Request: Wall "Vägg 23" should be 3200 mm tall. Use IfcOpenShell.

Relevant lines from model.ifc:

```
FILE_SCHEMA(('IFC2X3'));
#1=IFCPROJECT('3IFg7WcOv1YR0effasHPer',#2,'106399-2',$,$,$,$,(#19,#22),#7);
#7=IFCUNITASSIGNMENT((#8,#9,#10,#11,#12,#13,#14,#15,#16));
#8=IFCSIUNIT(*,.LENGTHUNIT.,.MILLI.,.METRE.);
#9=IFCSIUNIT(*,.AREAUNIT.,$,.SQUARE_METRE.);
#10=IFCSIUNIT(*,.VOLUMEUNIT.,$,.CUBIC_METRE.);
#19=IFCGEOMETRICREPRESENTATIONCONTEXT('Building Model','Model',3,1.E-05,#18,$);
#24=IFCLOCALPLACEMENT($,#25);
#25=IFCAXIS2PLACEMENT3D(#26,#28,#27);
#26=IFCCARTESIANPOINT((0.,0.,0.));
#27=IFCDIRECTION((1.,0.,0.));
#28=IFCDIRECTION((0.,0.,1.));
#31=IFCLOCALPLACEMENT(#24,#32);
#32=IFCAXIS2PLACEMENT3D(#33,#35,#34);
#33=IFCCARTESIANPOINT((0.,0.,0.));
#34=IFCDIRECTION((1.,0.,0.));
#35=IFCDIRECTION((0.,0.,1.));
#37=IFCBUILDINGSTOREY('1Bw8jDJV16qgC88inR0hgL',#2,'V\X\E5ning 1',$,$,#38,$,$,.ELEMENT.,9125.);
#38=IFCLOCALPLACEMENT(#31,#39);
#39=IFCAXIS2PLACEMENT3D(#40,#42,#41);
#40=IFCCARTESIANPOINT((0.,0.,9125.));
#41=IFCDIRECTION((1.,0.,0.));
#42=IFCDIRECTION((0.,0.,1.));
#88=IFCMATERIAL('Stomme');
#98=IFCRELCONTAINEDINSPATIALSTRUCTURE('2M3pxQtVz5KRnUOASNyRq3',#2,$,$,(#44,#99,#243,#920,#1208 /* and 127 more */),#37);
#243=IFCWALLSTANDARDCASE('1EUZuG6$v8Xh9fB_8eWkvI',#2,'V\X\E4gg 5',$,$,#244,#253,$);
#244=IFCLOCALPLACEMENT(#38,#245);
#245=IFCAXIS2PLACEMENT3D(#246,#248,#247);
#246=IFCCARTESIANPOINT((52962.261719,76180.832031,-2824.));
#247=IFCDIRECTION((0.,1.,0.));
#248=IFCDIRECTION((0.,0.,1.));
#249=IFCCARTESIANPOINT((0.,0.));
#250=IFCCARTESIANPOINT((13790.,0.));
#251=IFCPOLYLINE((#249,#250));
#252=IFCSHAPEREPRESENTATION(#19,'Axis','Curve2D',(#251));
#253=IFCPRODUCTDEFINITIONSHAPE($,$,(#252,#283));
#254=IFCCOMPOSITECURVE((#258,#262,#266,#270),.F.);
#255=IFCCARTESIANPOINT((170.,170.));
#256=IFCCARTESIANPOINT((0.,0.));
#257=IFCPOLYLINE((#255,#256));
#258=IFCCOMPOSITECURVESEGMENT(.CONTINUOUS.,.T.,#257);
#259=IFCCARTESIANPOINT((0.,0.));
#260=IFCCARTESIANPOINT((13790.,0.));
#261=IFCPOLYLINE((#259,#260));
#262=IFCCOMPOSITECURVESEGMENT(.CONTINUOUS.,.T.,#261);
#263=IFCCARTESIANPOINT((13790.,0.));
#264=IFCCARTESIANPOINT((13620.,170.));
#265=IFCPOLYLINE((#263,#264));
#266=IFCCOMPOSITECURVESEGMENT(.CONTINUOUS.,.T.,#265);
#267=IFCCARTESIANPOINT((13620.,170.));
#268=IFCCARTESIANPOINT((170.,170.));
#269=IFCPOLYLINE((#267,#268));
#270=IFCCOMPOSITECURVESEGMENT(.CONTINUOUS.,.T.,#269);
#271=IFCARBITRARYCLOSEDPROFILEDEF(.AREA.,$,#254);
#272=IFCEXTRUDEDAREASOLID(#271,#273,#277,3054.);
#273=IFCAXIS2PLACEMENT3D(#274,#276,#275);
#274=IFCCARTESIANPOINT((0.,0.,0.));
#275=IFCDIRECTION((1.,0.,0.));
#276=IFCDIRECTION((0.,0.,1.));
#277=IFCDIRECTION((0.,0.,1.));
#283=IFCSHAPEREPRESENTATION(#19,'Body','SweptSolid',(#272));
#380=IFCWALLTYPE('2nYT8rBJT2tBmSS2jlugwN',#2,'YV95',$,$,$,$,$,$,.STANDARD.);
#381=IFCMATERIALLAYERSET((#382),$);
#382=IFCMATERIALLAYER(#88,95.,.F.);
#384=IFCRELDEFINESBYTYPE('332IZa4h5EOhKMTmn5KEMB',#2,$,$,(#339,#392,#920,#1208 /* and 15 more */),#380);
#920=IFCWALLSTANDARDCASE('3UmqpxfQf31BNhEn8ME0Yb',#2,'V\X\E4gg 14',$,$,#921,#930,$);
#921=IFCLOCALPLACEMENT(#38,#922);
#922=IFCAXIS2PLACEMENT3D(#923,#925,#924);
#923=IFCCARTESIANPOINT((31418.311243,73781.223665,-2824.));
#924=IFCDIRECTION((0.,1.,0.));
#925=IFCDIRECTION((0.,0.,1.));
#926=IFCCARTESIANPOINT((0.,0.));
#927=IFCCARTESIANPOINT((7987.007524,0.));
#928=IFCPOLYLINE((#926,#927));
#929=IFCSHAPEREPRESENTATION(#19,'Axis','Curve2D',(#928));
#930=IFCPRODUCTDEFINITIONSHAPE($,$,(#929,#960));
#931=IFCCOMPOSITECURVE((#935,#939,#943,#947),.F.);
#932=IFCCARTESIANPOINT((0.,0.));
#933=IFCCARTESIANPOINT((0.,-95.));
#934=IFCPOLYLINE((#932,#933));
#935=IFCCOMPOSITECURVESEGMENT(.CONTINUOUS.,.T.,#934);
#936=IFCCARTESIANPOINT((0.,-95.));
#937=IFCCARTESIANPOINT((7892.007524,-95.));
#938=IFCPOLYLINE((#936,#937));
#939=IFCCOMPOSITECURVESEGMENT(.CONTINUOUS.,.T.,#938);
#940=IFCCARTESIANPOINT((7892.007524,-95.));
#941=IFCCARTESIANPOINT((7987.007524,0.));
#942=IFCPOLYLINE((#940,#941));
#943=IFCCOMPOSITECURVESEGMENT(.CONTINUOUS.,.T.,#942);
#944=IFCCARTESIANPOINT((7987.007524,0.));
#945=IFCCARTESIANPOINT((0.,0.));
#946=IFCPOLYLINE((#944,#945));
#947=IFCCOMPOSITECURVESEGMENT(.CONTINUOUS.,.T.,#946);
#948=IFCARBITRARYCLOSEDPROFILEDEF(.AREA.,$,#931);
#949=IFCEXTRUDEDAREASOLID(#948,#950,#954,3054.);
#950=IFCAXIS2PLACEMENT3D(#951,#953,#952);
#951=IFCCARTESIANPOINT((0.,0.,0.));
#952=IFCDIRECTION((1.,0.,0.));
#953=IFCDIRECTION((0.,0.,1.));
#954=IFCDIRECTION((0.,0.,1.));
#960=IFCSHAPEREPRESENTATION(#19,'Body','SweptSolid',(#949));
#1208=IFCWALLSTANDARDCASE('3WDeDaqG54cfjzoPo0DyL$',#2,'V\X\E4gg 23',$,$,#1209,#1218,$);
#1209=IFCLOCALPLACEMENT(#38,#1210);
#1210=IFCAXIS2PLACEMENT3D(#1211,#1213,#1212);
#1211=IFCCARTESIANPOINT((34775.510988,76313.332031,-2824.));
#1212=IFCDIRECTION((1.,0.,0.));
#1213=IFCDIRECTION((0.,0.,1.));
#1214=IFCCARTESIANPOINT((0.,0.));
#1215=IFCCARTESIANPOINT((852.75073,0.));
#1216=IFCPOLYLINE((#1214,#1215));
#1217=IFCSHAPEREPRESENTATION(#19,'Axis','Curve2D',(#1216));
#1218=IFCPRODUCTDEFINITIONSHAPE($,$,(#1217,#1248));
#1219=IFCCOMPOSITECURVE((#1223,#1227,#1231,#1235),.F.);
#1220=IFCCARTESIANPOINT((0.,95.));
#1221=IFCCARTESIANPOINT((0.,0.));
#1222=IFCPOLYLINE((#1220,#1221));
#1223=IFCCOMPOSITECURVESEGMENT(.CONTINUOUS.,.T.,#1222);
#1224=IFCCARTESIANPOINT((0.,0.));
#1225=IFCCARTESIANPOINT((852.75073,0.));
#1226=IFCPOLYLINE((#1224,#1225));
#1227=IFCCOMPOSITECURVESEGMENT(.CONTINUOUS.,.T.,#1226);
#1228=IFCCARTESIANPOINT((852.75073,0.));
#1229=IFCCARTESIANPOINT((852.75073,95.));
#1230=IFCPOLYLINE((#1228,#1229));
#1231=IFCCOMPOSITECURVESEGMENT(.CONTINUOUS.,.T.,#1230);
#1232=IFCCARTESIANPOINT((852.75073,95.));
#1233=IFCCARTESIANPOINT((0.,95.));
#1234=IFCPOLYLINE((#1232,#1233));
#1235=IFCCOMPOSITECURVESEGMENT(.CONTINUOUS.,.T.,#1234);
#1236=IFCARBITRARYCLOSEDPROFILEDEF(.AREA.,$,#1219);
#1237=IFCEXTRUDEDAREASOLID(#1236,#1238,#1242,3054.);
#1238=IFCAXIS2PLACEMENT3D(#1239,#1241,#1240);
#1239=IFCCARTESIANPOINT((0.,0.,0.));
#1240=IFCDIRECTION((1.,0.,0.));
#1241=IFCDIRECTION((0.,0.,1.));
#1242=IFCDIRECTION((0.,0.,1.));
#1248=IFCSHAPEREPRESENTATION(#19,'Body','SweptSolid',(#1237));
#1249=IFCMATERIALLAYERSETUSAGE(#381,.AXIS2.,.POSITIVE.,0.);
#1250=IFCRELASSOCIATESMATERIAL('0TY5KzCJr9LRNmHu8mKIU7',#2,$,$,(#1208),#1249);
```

```python
import ifcopenshell
import ifcopenshell.geom
import ifcopenshell.util.shape
import ifcopenshell.util.unit

model = ifcopenshell.open("model.ifc")
unit_scale = ifcopenshell.util.unit.calculate_unit_scale(model)
settings = ifcopenshell.geom.settings()


def volume(element):
    """Net volume in cubic metres, openings subtracted."""
    shape = ifcopenshell.geom.create_shape(settings, element)
    return ifcopenshell.util.shape.get_volume(shape.geometry)


wall = model.by_guid("3WDeDaqG54cfjzoPo0DyL$")
before = volume(wall)

body = next(r for r in wall.Representation.Representations if r.RepresentationIdentifier == "Body")
solid = body.Items[0]
old_height = solid.Depth
solid.Depth = 3.2 / unit_scale
after = volume(wall)

print(f"height {old_height:g} -> {solid.Depth:g}, volume {before:.3f} -> {after:.3f} m3")

model.write("model_rev.ifc")
```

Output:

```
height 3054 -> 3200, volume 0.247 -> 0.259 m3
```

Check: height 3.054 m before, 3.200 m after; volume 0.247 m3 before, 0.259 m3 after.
